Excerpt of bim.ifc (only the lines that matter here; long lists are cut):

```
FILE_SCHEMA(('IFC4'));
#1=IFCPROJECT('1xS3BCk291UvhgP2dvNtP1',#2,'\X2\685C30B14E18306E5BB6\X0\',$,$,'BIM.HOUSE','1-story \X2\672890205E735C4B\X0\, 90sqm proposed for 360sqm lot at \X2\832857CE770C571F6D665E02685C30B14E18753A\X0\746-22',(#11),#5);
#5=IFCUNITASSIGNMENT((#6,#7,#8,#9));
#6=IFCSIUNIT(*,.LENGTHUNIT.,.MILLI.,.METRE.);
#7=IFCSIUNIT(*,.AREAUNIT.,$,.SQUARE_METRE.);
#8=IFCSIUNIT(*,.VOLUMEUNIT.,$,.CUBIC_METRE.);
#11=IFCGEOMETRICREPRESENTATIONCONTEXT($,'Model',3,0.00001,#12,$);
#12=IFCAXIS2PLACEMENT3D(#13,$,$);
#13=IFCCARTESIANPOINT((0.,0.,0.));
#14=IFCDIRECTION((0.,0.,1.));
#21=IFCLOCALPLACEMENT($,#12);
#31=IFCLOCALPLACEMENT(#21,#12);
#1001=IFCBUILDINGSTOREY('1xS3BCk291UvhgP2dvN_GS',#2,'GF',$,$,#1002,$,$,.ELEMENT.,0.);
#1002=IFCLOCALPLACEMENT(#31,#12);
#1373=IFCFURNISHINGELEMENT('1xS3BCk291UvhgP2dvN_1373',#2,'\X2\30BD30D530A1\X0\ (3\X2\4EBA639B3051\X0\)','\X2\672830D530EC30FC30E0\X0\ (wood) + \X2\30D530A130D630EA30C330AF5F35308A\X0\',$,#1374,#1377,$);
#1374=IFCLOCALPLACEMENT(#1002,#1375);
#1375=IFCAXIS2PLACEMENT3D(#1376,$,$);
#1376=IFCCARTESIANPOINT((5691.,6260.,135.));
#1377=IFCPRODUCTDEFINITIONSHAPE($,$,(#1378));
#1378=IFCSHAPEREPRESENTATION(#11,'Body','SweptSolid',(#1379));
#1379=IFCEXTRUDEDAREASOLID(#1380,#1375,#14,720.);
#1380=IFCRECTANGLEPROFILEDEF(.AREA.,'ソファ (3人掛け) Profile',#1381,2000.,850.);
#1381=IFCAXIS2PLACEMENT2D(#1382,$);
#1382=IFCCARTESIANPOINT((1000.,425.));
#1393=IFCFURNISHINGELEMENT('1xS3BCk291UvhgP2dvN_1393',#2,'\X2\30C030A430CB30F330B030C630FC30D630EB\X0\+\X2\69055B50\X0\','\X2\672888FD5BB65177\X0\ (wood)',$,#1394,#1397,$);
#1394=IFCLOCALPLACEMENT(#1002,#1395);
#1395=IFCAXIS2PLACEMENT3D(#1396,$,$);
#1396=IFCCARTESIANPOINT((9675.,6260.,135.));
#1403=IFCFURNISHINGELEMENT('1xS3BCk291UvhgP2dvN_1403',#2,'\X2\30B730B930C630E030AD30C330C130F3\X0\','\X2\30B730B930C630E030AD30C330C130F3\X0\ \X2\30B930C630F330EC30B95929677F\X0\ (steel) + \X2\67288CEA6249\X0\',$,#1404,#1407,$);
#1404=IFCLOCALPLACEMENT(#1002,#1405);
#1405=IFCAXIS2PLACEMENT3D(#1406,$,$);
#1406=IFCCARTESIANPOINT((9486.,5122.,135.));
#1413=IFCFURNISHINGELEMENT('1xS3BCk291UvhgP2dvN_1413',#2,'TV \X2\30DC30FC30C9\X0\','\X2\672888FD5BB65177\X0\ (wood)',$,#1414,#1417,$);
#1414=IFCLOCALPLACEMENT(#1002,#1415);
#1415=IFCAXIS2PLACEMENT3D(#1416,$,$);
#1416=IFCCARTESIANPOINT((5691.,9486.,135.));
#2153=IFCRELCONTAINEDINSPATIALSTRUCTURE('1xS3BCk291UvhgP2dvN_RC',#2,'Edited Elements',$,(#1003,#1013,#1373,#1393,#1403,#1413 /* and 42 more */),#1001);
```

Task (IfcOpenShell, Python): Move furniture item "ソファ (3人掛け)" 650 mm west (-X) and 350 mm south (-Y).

```python
import ifcopenshell
import ifcopenshell.api.geometry
import ifcopenshell.util.placement

model = ifcopenshell.open("bim.ifc")

item = model.by_guid("1xS3BCk291UvhgP2dvN_1373")
matrix = ifcopenshell.util.placement.get_local_placement(item.ObjectPlacement)
matrix[0, 3] -= 650.0
matrix[1, 3] -= 350.0
ifcopenshell.api.geometry.edit_object_placement(model, product=item, matrix=matrix, is_si=False)

print(ifcopenshell.util.placement.get_local_placement(item.ObjectPlacement).round(3) + 0.0)

model.write("bim_edited.ifc")
```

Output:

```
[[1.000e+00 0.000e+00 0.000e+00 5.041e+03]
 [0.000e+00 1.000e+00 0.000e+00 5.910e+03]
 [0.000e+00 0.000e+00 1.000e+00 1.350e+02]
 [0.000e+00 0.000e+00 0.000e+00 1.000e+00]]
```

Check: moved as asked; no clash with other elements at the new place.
